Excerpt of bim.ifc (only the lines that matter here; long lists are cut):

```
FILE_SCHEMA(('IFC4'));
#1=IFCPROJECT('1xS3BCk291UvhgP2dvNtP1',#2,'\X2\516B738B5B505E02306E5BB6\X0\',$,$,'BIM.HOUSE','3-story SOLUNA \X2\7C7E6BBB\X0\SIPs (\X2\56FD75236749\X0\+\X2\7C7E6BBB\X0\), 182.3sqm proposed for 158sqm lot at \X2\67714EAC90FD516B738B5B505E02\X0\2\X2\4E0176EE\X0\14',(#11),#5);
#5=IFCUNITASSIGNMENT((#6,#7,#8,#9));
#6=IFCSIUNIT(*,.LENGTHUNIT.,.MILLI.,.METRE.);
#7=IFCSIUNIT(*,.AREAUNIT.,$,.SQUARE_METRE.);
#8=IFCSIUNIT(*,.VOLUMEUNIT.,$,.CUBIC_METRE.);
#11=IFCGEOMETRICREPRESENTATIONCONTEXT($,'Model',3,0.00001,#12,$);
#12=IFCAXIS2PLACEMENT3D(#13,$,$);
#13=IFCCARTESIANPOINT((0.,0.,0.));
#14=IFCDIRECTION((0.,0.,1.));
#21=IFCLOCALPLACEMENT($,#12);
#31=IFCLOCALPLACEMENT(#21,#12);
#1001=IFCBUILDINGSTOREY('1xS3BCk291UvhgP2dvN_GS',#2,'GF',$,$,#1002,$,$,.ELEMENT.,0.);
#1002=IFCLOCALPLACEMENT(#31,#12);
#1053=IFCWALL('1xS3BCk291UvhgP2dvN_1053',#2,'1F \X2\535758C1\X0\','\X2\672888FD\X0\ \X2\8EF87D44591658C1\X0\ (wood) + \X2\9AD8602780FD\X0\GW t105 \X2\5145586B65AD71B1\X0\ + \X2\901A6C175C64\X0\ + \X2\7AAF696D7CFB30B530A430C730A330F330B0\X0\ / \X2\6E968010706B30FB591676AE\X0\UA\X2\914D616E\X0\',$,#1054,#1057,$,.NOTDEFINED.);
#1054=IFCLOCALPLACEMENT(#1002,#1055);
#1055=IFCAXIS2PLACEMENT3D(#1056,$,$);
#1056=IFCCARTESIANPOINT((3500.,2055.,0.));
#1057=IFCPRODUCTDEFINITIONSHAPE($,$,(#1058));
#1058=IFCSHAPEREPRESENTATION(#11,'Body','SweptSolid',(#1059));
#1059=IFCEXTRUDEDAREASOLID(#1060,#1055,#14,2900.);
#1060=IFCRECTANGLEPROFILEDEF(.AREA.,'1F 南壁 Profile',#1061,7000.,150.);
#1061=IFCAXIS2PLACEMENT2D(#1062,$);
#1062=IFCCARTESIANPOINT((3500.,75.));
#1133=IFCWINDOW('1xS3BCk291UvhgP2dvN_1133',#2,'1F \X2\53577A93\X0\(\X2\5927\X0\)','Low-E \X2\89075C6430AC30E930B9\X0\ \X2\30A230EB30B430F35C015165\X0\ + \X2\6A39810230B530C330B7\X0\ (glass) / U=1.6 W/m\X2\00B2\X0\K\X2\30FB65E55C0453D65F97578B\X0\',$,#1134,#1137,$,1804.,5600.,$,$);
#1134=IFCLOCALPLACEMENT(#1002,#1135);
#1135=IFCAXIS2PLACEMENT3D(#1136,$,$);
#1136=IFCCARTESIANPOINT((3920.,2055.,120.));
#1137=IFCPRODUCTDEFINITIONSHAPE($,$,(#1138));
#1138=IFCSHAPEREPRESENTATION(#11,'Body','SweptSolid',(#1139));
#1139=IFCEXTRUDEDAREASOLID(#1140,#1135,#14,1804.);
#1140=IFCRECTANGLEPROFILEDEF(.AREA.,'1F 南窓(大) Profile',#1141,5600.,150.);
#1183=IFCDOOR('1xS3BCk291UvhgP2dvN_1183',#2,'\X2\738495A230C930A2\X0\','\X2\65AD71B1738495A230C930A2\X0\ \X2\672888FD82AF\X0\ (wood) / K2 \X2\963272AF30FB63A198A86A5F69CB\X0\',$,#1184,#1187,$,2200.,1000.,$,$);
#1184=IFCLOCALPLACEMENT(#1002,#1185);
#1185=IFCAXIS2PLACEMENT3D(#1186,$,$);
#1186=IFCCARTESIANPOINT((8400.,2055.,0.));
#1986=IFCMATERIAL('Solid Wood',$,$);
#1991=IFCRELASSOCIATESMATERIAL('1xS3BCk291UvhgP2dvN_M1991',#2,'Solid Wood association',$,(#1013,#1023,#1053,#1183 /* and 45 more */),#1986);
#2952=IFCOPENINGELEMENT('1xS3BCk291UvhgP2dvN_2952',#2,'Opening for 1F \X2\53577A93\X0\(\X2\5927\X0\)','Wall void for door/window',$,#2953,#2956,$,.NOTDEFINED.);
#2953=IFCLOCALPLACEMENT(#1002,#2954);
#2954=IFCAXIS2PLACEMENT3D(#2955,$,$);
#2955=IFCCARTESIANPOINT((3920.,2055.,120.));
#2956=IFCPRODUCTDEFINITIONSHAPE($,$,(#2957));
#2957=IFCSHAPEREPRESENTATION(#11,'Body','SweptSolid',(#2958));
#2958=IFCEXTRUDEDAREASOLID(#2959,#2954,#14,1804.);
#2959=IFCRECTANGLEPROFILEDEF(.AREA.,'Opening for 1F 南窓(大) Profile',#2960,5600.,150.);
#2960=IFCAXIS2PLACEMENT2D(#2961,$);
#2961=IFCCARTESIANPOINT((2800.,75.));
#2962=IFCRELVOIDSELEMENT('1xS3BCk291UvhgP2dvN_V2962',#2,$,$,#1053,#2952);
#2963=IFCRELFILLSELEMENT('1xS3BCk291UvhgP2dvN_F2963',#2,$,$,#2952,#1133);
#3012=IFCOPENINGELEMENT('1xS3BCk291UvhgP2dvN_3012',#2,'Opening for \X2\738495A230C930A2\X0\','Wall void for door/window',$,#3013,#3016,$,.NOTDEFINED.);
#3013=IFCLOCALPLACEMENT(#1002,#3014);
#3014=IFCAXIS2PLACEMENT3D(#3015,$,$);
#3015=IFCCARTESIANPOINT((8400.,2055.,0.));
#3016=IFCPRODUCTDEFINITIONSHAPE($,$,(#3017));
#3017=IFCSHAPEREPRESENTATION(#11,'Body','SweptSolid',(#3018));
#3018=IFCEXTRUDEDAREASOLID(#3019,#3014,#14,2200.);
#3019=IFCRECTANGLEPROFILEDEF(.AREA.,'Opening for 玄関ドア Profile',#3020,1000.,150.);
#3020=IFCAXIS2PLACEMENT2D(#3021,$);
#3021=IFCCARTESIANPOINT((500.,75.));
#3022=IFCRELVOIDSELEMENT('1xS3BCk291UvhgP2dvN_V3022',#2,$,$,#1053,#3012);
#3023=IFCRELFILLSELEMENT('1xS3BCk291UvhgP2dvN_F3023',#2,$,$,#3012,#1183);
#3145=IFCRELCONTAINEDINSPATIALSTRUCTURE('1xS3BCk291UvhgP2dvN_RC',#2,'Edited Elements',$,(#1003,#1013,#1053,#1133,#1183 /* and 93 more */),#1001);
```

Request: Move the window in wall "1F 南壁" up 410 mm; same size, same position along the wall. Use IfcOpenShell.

```python
import numpy as np
import ifcopenshell
import ifcopenshell.api.geometry
import ifcopenshell.util.placement
import ifcopenshell.util.unit

model = ifcopenshell.open("bim.ifc")
unit_scale = ifcopenshell.util.unit.calculate_unit_scale(model)

window = model.by_guid("1xS3BCk291UvhgP2dvN_1133")
opening = window.FillsVoids[0].RelatingOpeningElement
dz = 410.0

shift = np.array([0.0, 0.0, dz])
# The window is not placed relative to its opening, so move both.
for product in (opening, window):
    matrix = ifcopenshell.util.placement.get_local_placement(product.ObjectPlacement)
    matrix[:3, 3] += shift
    ifcopenshell.api.geometry.edit_object_placement(model, product=product, matrix=matrix, is_si=False)

print(f"moved by {dz * unit_scale:+.3f} m")

model.write("bim_v2.ifc")
```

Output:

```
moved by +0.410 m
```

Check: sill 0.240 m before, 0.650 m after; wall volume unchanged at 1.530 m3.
